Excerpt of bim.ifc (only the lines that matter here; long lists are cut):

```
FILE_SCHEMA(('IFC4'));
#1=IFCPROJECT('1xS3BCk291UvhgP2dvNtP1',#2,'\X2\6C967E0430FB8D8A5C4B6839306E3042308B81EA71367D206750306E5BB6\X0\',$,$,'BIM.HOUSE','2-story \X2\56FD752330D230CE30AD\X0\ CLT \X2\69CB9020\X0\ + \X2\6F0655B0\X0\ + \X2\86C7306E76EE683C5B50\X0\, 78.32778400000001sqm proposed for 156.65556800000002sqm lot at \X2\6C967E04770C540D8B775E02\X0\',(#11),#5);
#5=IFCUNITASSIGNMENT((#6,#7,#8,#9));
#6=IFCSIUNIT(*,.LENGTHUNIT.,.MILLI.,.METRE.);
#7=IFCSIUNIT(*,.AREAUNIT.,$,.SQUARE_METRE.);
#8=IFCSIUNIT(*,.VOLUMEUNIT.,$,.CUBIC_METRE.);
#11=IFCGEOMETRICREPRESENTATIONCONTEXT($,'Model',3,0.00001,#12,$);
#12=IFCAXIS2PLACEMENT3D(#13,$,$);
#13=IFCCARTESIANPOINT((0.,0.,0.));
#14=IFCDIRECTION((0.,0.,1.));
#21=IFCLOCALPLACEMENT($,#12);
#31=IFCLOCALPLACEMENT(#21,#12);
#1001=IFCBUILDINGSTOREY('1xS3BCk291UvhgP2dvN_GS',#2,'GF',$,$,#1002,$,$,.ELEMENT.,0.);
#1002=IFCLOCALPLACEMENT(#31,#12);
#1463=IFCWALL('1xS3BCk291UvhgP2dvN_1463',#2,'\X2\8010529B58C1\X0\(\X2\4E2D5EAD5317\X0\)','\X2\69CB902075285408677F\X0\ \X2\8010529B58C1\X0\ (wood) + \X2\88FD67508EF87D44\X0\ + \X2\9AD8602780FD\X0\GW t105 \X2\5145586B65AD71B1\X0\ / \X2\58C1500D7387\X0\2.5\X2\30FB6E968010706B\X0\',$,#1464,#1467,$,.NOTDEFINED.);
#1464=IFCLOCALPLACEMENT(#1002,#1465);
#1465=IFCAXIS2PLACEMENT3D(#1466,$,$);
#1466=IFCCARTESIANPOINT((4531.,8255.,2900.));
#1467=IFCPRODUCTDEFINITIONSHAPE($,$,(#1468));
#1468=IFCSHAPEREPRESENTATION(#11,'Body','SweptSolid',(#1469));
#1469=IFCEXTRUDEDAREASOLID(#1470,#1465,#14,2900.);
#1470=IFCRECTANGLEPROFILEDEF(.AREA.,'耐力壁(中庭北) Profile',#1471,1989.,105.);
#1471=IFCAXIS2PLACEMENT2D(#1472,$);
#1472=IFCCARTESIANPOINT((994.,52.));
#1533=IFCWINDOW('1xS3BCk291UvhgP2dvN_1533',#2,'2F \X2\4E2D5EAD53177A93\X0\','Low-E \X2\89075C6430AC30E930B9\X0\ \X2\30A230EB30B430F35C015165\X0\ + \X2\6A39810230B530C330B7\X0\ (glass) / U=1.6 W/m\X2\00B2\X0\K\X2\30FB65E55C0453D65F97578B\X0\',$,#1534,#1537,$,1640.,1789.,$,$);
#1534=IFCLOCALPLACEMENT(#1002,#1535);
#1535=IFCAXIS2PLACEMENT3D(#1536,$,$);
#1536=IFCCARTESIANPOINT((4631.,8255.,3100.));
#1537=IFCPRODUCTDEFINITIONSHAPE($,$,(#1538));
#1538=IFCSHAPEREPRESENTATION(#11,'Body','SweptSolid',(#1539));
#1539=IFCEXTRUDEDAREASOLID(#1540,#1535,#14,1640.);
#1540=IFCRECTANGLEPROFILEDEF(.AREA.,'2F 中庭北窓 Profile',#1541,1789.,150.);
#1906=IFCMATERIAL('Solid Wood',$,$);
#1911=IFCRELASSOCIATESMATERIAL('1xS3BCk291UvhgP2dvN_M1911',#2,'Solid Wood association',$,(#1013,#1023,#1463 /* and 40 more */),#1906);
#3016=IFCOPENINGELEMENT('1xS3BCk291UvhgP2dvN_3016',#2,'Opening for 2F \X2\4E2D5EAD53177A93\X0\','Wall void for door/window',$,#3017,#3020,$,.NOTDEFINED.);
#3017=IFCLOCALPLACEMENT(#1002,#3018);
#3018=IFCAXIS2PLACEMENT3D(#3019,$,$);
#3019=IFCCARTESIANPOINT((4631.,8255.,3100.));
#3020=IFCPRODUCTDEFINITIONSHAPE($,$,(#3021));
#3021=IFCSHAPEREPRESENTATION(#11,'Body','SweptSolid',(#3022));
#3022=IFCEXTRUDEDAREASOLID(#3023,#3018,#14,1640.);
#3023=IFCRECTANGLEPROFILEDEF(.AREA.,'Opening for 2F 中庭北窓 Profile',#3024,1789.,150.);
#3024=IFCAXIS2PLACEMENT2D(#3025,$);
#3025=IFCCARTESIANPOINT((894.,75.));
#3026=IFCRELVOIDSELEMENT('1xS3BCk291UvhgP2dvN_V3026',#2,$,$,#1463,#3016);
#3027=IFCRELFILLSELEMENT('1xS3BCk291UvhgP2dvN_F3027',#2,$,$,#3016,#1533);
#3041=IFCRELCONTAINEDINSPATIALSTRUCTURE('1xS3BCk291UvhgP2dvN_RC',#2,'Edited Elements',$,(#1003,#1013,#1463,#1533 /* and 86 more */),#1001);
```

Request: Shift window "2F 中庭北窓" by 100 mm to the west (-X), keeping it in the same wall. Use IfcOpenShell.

```python
import ifcopenshell
import ifcopenshell.api.geometry
import ifcopenshell.util.placement
import ifcopenshell.util.unit

model = ifcopenshell.open("bim.ifc")
unit_scale = ifcopenshell.util.unit.calculate_unit_scale(model)

window = model.by_guid("1xS3BCk291UvhgP2dvN_1533")
opening = window.FillsVoids[0].RelatingOpeningElement
wall = opening.VoidsElements[0].RelatingBuildingElement

wall_matrix = ifcopenshell.util.placement.get_local_placement(wall.ObjectPlacement)
shift = wall_matrix[:3, 0] * -0.1 / unit_scale
before = ifcopenshell.util.placement.get_local_placement(window.ObjectPlacement)[:3, 3].copy()

# The window is not placed relative to its opening, so move both.
for product in (opening, window):
    matrix = ifcopenshell.util.placement.get_local_placement(product.ObjectPlacement)
    matrix[:3, 3] += shift
    ifcopenshell.api.geometry.edit_object_placement(model, product=product, matrix=matrix, is_si=False)

after = ifcopenshell.util.placement.get_local_placement(window.ObjectPlacement)[:3, 3]
print("window moved by", (after - before).round(3) + 0.0)

model.write("bim_v2.ifc")
```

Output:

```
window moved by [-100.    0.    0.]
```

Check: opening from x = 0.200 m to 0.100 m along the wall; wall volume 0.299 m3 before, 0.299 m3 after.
